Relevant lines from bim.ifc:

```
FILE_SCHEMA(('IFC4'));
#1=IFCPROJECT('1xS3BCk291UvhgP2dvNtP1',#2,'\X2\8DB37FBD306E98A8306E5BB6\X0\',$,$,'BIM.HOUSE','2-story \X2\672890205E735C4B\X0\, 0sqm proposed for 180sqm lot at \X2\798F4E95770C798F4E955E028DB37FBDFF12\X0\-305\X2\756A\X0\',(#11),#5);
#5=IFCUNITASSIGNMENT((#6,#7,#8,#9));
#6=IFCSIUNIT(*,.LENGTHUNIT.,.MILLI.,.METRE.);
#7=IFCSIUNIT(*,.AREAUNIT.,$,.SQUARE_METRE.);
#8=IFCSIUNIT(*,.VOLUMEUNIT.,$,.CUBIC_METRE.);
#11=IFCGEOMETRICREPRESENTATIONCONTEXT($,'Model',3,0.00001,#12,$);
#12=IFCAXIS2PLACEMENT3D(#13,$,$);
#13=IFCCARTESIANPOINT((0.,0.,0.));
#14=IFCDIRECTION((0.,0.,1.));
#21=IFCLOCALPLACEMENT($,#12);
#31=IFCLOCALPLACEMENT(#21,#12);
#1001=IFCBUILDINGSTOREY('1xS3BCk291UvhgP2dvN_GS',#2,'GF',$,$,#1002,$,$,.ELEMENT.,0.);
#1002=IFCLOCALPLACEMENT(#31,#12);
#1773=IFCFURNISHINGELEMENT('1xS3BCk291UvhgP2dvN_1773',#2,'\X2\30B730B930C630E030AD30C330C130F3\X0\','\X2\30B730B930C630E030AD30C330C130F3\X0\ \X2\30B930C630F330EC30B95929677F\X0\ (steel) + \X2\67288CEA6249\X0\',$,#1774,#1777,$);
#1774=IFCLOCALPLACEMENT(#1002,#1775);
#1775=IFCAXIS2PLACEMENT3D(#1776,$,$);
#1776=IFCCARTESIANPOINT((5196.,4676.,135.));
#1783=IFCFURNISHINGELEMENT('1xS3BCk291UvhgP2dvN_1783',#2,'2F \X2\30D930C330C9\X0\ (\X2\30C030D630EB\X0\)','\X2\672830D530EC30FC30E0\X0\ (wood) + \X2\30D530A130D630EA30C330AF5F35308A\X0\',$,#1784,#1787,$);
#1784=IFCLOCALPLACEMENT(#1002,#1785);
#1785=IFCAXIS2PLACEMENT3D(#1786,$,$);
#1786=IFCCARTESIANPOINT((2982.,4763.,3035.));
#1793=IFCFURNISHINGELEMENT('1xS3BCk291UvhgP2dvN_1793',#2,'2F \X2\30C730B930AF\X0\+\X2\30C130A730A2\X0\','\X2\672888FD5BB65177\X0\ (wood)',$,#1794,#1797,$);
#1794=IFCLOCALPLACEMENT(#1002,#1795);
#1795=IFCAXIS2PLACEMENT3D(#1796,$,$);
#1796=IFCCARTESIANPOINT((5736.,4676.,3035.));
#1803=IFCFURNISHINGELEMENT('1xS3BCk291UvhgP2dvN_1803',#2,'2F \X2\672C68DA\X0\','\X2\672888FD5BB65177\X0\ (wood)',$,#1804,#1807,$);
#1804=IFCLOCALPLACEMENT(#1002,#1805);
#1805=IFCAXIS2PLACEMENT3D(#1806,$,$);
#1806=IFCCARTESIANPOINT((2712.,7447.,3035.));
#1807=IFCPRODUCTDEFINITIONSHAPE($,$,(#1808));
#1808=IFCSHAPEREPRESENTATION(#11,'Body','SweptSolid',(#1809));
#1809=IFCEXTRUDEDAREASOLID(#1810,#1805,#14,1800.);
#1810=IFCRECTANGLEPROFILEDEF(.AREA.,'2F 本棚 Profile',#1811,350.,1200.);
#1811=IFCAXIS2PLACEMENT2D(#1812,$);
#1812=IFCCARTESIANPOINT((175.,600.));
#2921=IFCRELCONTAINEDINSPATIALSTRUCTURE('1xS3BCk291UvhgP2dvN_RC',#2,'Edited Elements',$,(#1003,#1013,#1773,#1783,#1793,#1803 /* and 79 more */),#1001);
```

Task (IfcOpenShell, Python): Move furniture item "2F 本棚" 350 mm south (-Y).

```python
import ifcopenshell
import ifcopenshell.api.geometry
import ifcopenshell.util.placement

model = ifcopenshell.open("bim.ifc")

item = model.by_id(1803)
matrix = ifcopenshell.util.placement.get_local_placement(item.ObjectPlacement)
matrix[1, 3] -= 350.0
ifcopenshell.api.geometry.edit_object_placement(model, product=item, matrix=matrix, is_si=False)

print(ifcopenshell.util.placement.get_local_placement(item.ObjectPlacement).round(3) + 0.0)

model.write("bim-out.ifc")
```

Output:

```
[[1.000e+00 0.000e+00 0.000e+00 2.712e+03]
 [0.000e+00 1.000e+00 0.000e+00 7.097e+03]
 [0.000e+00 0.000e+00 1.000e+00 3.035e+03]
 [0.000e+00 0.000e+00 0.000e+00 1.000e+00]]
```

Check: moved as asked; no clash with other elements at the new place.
